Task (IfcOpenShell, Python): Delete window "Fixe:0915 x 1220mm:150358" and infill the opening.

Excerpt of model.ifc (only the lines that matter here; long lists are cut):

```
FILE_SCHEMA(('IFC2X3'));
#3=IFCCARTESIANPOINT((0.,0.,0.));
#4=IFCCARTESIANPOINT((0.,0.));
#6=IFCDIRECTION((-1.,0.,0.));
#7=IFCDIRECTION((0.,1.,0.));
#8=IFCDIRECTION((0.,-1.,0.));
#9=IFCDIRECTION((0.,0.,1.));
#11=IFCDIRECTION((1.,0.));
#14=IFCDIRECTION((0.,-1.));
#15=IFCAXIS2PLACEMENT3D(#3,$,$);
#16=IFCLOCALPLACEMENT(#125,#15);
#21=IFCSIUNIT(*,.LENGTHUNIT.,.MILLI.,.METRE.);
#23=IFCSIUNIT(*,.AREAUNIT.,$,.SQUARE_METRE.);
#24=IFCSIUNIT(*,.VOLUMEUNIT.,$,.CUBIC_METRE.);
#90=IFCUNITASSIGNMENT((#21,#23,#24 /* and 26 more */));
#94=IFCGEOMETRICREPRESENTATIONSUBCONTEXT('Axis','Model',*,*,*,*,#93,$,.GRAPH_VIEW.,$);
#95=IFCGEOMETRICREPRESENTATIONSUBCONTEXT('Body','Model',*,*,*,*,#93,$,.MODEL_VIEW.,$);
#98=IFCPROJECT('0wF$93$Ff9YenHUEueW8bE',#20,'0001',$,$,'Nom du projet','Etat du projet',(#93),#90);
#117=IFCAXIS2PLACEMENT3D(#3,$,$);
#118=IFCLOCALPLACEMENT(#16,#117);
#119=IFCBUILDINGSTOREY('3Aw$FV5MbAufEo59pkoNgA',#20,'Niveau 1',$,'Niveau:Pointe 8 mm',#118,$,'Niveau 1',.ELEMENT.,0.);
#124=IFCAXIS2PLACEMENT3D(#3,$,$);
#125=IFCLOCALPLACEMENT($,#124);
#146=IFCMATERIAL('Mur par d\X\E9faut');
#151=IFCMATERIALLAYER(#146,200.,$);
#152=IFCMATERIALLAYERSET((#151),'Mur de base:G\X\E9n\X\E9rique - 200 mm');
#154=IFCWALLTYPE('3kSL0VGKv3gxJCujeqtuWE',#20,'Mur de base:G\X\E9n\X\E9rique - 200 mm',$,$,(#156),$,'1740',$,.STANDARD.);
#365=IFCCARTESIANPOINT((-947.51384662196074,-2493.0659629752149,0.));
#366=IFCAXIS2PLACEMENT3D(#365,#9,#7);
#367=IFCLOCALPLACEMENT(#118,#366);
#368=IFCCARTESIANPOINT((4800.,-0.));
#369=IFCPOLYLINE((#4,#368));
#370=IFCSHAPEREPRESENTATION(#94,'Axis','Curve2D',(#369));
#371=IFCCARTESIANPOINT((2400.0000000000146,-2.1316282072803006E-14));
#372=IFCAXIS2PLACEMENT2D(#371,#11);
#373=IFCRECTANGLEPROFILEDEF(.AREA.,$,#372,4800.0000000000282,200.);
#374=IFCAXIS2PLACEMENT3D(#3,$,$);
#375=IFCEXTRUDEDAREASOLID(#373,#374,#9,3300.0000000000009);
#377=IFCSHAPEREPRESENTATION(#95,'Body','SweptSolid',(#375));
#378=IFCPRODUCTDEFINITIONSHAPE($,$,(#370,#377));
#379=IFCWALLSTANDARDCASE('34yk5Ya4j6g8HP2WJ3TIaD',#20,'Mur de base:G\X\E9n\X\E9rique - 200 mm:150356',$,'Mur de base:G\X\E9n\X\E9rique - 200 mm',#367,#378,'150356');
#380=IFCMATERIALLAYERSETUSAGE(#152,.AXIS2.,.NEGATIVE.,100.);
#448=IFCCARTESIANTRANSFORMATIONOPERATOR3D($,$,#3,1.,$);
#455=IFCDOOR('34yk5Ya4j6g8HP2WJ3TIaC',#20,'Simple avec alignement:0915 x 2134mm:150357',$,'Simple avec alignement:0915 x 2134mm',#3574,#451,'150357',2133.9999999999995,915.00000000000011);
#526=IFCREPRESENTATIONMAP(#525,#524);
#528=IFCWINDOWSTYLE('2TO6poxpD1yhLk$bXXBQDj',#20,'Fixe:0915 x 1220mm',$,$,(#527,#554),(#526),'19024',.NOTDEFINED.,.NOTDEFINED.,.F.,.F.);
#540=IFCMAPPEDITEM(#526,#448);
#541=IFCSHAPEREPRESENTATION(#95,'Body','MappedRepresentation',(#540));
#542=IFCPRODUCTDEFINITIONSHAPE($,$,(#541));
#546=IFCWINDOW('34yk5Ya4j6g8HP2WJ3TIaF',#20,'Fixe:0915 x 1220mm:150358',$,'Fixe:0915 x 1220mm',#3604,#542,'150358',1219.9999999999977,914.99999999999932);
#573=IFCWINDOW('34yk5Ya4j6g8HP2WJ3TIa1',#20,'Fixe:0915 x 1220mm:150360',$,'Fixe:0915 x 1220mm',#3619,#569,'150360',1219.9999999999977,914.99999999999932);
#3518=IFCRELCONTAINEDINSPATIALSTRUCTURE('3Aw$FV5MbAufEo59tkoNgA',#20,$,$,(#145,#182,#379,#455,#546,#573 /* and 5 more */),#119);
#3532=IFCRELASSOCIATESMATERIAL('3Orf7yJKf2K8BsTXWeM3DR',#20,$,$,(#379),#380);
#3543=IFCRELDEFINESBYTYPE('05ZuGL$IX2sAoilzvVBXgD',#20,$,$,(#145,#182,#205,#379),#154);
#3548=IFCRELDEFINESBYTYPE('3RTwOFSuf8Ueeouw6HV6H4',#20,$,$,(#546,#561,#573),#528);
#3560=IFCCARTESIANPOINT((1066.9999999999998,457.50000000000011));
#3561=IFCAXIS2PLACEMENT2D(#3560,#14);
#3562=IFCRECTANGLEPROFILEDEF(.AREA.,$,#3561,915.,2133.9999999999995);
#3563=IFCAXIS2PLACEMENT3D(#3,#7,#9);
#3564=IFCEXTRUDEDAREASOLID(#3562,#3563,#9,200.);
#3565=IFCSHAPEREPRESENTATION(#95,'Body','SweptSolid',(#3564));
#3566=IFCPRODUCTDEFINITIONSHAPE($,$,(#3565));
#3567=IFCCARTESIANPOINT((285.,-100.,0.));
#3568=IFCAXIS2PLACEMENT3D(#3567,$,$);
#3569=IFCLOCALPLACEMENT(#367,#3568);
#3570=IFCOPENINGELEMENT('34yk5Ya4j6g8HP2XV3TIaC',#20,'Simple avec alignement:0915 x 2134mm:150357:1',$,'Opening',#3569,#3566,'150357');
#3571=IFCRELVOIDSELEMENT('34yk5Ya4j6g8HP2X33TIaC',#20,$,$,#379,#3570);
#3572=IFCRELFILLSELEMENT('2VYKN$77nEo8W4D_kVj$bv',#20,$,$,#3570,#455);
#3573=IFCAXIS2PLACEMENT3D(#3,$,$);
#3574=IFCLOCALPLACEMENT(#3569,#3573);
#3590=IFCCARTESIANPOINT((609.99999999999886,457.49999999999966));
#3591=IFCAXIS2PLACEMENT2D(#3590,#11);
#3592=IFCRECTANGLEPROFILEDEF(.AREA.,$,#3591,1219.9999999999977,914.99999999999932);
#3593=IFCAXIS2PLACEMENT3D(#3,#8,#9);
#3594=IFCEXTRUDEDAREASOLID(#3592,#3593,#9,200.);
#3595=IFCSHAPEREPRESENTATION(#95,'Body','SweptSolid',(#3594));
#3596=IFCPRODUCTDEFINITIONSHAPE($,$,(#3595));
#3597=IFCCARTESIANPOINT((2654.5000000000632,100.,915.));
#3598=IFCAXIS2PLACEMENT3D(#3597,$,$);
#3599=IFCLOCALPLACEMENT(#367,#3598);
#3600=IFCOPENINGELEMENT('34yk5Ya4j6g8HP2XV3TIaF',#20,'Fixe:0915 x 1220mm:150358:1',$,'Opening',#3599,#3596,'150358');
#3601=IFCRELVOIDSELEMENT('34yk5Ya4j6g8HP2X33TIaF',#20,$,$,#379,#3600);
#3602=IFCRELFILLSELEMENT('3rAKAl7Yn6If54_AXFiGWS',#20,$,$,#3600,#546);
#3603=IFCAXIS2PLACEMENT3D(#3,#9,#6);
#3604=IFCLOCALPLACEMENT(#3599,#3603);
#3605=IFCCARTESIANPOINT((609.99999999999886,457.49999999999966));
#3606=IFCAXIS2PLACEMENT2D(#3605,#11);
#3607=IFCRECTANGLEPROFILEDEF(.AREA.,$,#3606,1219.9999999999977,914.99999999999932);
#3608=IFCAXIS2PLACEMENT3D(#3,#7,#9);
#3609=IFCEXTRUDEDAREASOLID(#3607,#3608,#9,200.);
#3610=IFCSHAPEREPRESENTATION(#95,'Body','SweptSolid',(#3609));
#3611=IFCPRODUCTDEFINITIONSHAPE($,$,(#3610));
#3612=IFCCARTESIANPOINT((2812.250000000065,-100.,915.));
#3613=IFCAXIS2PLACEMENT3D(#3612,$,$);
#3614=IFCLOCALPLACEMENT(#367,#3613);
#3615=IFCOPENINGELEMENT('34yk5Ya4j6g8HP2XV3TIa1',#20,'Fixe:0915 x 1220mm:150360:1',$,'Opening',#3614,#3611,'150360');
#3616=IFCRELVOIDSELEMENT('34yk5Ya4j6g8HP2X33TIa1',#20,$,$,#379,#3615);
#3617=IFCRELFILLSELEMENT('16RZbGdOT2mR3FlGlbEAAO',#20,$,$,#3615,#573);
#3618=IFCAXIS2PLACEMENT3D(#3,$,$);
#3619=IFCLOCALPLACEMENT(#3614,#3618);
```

```python
import ifcopenshell
import ifcopenshell.api.feature
import ifcopenshell.api.root
import ifcopenshell.geom
import ifcopenshell.util.shape

model = ifcopenshell.open("model.ifc")
settings = ifcopenshell.geom.settings()


def volume(element):
    """Net volume in cubic metres, openings subtracted."""
    shape = ifcopenshell.geom.create_shape(settings, element)
    return ifcopenshell.util.shape.get_volume(shape.geometry)


window = model.by_guid("34yk5Ya4j6g8HP2WJ3TIaF")
opening = window.FillsVoids[0].RelatingOpeningElement
wall = opening.VoidsElements[0].RelatingBuildingElement
before = volume(wall)

ifcopenshell.api.root.remove_product(model, product=window)
ifcopenshell.api.feature.remove_feature(model, feature=opening)

after = volume(wall)

print(f"wall volume {before:.3f} -> {after:.3f} m3")

model.write("model_v2.ifc")
```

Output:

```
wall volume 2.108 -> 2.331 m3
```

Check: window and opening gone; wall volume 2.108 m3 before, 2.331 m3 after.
